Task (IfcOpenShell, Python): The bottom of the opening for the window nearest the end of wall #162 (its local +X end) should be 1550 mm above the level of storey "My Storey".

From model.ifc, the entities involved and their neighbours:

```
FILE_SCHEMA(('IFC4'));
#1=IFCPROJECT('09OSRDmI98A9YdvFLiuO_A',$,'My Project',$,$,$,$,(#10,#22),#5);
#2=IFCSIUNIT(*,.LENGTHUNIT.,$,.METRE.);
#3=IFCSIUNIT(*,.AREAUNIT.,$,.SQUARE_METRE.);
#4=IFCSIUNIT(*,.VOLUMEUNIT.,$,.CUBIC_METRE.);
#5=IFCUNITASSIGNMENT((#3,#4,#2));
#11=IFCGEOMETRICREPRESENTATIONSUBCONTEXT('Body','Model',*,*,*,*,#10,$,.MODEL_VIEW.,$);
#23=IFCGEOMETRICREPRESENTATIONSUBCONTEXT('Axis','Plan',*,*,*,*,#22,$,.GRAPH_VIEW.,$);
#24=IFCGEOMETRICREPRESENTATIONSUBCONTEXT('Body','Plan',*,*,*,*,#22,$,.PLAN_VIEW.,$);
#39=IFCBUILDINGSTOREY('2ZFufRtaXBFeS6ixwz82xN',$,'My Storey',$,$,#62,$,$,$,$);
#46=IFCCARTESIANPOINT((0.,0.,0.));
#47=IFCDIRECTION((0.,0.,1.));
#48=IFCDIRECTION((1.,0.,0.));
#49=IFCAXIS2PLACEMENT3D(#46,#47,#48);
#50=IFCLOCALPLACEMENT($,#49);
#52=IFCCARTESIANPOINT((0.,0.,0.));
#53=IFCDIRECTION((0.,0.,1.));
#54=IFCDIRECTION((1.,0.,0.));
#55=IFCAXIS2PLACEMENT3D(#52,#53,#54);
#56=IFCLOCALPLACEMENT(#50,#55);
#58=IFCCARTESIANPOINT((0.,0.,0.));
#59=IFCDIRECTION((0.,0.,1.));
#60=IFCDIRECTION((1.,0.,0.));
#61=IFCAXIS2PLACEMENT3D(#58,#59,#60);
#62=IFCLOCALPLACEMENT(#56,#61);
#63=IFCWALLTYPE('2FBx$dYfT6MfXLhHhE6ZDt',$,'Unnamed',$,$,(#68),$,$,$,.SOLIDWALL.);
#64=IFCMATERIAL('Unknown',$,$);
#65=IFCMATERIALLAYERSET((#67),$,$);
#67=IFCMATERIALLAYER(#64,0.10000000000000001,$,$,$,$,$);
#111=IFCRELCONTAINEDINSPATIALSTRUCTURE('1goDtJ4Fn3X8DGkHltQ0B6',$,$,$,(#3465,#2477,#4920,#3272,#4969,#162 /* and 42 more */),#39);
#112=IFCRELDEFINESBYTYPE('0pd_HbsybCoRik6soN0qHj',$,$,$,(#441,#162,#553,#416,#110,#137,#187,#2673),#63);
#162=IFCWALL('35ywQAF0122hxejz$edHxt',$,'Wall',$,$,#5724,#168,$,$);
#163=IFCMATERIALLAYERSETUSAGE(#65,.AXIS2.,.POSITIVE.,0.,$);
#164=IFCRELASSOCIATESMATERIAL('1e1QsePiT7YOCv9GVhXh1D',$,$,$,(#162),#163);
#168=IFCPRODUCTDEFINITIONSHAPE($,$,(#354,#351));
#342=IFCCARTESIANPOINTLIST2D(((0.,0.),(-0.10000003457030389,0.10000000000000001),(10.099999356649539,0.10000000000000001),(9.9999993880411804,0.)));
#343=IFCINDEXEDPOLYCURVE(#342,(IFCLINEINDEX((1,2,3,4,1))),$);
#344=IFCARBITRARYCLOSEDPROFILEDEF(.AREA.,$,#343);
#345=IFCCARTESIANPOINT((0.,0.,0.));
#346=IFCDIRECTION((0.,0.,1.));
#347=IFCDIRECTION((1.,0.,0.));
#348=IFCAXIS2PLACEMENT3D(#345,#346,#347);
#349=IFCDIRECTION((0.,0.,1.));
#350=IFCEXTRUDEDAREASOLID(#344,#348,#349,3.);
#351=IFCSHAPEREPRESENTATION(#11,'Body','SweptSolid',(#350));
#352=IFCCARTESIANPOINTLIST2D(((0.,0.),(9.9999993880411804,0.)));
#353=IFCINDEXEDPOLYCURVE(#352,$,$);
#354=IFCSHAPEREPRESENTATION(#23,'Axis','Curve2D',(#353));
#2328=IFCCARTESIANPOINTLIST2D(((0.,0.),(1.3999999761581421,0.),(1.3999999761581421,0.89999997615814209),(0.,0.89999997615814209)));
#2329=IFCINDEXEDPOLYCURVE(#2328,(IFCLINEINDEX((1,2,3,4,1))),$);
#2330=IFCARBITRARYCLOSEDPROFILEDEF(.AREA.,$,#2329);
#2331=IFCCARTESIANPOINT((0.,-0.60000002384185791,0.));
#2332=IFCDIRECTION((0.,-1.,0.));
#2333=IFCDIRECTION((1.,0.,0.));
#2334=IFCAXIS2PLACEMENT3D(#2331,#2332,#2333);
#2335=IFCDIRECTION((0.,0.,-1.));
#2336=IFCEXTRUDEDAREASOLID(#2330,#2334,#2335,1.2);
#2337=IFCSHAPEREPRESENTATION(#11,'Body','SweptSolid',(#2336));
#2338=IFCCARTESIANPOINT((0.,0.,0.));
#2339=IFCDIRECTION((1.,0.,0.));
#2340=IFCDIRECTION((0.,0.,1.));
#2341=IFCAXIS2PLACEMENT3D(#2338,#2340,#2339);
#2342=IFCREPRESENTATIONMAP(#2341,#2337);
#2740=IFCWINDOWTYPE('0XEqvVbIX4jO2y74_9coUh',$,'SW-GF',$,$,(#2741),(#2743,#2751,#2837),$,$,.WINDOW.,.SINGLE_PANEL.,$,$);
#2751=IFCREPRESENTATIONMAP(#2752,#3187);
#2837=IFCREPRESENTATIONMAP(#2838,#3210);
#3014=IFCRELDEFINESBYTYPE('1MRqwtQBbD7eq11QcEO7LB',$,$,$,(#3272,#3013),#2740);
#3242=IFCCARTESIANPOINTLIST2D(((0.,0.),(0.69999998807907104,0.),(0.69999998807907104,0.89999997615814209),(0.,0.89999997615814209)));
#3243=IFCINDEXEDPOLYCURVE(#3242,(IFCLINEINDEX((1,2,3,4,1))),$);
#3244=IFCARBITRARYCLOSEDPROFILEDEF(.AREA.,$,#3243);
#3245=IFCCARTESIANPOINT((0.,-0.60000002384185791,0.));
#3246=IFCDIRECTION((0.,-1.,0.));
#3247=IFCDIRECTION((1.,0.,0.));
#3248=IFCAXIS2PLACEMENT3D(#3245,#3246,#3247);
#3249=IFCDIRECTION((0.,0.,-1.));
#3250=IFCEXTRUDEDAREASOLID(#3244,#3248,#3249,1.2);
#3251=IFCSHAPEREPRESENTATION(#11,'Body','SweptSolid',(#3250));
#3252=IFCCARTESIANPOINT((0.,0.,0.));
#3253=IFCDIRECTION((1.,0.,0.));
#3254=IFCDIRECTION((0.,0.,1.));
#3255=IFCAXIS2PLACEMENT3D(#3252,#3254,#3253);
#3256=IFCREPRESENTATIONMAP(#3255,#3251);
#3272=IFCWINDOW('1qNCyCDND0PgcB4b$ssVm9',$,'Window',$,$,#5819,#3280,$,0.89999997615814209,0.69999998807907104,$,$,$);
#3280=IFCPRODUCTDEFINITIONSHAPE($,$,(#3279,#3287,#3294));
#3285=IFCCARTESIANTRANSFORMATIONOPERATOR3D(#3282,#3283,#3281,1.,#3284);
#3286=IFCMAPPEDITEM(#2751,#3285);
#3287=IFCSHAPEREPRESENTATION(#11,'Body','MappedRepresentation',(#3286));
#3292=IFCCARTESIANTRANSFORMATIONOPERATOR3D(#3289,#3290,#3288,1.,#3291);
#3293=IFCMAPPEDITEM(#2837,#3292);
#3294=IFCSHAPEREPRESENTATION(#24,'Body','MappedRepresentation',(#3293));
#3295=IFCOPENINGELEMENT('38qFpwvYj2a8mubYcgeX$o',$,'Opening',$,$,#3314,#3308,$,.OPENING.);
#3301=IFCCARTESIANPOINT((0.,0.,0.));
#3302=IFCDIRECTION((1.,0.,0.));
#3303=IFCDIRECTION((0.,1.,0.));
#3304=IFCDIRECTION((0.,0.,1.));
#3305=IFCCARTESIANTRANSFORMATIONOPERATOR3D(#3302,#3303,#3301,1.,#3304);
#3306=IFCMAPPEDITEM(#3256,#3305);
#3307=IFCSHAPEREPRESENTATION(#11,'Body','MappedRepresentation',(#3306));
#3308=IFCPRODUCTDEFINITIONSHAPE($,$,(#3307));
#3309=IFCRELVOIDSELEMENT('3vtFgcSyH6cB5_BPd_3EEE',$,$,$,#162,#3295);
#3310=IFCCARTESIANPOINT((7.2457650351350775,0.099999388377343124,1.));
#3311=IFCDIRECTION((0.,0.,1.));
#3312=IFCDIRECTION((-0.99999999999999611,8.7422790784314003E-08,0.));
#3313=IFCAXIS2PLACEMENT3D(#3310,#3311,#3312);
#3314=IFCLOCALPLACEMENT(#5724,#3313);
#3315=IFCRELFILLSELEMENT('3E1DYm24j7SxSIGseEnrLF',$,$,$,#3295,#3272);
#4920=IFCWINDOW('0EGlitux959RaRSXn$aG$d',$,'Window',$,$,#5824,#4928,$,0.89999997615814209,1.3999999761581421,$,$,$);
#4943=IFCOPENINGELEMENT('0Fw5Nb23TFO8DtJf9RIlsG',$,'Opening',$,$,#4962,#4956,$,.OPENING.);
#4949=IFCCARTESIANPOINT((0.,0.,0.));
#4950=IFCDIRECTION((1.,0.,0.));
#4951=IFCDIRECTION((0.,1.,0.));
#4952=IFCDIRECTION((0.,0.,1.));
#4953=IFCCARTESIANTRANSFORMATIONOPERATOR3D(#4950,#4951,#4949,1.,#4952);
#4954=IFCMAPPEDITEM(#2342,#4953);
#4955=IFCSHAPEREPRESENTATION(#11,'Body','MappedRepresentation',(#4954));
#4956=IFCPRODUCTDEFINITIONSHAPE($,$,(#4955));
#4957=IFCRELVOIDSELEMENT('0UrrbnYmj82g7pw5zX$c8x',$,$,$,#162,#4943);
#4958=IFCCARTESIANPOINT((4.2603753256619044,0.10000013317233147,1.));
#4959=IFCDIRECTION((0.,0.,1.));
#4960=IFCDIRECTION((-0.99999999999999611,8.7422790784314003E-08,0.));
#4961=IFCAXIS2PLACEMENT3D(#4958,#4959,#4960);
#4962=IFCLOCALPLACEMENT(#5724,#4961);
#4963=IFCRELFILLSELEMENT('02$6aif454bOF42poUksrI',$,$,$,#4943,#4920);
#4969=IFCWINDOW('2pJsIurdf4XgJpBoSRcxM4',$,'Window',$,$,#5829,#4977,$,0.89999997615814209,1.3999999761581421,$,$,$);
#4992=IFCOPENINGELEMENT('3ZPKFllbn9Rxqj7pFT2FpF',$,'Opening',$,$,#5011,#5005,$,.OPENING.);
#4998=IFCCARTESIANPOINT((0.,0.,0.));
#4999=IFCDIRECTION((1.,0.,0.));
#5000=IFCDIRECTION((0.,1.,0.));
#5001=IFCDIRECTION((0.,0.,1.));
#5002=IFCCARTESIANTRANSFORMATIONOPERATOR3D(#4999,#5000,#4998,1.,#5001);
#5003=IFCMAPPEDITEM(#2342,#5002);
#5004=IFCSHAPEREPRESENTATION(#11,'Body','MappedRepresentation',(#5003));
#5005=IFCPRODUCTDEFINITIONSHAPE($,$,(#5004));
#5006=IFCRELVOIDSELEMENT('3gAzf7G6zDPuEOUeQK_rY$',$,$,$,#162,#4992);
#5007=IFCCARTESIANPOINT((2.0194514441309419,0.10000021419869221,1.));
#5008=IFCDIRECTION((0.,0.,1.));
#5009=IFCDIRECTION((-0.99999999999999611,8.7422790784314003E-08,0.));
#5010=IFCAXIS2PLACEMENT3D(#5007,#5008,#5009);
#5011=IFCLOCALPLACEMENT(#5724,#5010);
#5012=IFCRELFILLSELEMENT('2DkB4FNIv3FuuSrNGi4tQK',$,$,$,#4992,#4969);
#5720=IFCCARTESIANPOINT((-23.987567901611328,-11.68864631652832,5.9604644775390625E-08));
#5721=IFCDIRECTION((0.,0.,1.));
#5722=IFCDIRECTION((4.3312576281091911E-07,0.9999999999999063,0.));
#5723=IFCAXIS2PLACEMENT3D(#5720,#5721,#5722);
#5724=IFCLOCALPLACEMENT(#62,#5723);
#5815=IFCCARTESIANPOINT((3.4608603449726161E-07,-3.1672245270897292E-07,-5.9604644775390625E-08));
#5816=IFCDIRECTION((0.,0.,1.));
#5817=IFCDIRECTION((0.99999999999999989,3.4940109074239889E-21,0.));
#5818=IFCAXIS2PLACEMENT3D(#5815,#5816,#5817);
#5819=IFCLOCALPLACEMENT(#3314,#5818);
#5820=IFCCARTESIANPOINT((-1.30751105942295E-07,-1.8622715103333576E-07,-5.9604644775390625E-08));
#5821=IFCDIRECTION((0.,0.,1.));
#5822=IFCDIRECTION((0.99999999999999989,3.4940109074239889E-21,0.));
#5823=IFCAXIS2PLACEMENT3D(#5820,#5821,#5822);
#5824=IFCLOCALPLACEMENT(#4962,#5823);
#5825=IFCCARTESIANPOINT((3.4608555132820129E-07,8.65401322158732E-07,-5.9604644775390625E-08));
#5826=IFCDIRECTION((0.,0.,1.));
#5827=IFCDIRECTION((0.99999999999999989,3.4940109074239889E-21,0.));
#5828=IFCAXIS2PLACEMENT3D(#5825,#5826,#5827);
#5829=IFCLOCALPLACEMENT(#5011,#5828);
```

```python
import numpy as np
import ifcopenshell
import ifcopenshell.api.geometry
import ifcopenshell.geom
import ifcopenshell.util.element
import ifcopenshell.util.placement
import ifcopenshell.util.shape
import ifcopenshell.util.unit

model = ifcopenshell.open("model.ifc")
unit_scale = ifcopenshell.util.unit.calculate_unit_scale(model)

window = model.by_id(3272)
opening = window.FillsVoids[0].RelatingOpeningElement
storey = ifcopenshell.util.element.get_container(window, ifc_class="IfcBuildingStorey")
level = ifcopenshell.util.placement.get_local_placement(storey.ObjectPlacement)[2, 3]

# The opening's origin need not be at the sill, so measure its lowest point.
shape = ifcopenshell.geom.create_shape(ifcopenshell.geom.settings(), opening)
bottom = ifcopenshell.util.shape.get_shape_bottom_elevation(shape, shape.geometry) / unit_scale
dz = level + 1.55 - bottom

shift = np.array([0.0, 0.0, dz])
# The window is placed relative to its opening, so it follows when the opening moves.
matrix = ifcopenshell.util.placement.get_local_placement(opening.ObjectPlacement)
matrix[:3, 3] += shift
ifcopenshell.api.geometry.edit_object_placement(
    model, product=opening, matrix=matrix, is_si=False, should_transform_children=True
)

print(f"moved by {dz * unit_scale:+.3f} m")

model.write("model-out.ifc")
```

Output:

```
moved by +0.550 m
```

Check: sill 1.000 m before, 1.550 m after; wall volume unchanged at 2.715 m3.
